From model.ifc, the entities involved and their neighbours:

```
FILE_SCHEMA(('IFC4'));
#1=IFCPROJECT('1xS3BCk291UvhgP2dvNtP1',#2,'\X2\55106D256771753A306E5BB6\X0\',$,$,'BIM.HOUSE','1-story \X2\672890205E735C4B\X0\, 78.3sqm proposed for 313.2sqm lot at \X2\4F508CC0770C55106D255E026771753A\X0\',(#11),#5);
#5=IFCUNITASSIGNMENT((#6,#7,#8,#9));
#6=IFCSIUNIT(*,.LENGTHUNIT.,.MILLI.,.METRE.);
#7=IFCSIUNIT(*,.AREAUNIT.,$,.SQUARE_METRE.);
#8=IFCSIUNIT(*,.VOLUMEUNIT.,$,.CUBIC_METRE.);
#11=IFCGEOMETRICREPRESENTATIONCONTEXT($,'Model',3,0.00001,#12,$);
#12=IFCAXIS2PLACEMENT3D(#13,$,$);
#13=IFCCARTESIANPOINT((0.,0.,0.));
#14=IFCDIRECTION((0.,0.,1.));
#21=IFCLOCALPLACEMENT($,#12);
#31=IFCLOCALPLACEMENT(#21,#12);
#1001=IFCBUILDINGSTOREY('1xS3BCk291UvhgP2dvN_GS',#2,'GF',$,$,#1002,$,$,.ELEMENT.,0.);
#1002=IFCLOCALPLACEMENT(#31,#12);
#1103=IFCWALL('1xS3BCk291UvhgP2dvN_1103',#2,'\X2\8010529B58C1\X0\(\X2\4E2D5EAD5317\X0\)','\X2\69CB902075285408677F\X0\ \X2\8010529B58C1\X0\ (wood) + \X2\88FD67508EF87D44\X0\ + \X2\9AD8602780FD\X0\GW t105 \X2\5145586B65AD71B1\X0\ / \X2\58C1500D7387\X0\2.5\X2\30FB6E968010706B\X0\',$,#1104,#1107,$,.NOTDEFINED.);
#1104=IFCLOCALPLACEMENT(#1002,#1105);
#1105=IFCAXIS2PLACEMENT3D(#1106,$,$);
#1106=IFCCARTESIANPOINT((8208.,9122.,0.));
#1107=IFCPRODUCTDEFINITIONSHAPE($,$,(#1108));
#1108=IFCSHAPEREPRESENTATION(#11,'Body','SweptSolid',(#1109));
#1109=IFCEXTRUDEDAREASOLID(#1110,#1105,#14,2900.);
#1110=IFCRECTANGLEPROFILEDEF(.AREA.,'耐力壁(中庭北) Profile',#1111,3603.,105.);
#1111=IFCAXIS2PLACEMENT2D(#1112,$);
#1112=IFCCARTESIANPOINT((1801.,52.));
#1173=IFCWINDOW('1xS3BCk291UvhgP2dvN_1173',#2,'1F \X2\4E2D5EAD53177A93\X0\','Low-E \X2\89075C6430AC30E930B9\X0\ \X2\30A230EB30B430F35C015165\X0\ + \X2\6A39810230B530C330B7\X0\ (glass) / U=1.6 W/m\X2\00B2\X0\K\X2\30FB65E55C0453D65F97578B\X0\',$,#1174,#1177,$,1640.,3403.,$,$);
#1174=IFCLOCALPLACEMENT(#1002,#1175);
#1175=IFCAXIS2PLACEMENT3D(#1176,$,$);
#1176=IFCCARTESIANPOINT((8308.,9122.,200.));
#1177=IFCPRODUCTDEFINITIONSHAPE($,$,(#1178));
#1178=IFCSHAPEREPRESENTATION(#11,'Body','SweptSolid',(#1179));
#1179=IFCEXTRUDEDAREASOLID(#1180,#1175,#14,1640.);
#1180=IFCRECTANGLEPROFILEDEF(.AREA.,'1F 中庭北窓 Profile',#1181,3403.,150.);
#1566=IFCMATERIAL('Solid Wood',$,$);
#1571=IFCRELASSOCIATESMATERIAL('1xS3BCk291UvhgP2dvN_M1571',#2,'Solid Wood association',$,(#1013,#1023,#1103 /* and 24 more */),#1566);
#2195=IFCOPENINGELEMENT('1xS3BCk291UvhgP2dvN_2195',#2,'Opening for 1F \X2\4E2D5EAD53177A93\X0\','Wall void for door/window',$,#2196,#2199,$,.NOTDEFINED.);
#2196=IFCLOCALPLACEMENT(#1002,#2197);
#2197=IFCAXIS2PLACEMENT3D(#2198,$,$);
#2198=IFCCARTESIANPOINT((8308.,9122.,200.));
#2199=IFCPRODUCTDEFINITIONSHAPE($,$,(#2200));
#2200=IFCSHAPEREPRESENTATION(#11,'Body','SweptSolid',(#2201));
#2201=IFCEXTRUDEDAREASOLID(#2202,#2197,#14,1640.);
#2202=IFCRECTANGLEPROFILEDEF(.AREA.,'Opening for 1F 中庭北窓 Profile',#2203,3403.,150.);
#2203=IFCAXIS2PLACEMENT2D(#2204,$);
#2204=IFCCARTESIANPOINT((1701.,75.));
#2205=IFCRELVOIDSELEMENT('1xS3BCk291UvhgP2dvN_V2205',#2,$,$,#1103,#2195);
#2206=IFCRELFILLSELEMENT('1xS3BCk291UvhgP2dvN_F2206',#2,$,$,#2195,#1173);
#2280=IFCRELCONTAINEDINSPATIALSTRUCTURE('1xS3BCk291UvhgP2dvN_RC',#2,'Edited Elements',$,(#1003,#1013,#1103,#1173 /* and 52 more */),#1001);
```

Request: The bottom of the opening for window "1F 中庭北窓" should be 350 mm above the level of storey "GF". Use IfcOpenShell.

```python
import numpy as np
import ifcopenshell
import ifcopenshell.api.geometry
import ifcopenshell.geom
import ifcopenshell.util.element
import ifcopenshell.util.placement
import ifcopenshell.util.shape
import ifcopenshell.util.unit

model = ifcopenshell.open("model.ifc")
unit_scale = ifcopenshell.util.unit.calculate_unit_scale(model)

window = model.by_guid("1xS3BCk291UvhgP2dvN_1173")
opening = window.FillsVoids[0].RelatingOpeningElement
storey = ifcopenshell.util.element.get_container(window, ifc_class="IfcBuildingStorey")
level = ifcopenshell.util.placement.get_local_placement(storey.ObjectPlacement)[2, 3]

# The opening's origin need not be at the sill, so measure its lowest point.
shape = ifcopenshell.geom.create_shape(ifcopenshell.geom.settings(), opening)
bottom = ifcopenshell.util.shape.get_shape_bottom_elevation(shape, shape.geometry) / unit_scale
dz = level + 0.35 / unit_scale - bottom

shift = np.array([0.0, 0.0, dz])
# The window is not placed relative to its opening, so move both.
for product in (opening, window):
    matrix = ifcopenshell.util.placement.get_local_placement(product.ObjectPlacement)
    matrix[:3, 3] += shift
    ifcopenshell.api.geometry.edit_object_placement(model, product=product, matrix=matrix, is_si=False)

print(f"moved by {dz * unit_scale:+.3f} m")

model.write("model-out.ifc")
```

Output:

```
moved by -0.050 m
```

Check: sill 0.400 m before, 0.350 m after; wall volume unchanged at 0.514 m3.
